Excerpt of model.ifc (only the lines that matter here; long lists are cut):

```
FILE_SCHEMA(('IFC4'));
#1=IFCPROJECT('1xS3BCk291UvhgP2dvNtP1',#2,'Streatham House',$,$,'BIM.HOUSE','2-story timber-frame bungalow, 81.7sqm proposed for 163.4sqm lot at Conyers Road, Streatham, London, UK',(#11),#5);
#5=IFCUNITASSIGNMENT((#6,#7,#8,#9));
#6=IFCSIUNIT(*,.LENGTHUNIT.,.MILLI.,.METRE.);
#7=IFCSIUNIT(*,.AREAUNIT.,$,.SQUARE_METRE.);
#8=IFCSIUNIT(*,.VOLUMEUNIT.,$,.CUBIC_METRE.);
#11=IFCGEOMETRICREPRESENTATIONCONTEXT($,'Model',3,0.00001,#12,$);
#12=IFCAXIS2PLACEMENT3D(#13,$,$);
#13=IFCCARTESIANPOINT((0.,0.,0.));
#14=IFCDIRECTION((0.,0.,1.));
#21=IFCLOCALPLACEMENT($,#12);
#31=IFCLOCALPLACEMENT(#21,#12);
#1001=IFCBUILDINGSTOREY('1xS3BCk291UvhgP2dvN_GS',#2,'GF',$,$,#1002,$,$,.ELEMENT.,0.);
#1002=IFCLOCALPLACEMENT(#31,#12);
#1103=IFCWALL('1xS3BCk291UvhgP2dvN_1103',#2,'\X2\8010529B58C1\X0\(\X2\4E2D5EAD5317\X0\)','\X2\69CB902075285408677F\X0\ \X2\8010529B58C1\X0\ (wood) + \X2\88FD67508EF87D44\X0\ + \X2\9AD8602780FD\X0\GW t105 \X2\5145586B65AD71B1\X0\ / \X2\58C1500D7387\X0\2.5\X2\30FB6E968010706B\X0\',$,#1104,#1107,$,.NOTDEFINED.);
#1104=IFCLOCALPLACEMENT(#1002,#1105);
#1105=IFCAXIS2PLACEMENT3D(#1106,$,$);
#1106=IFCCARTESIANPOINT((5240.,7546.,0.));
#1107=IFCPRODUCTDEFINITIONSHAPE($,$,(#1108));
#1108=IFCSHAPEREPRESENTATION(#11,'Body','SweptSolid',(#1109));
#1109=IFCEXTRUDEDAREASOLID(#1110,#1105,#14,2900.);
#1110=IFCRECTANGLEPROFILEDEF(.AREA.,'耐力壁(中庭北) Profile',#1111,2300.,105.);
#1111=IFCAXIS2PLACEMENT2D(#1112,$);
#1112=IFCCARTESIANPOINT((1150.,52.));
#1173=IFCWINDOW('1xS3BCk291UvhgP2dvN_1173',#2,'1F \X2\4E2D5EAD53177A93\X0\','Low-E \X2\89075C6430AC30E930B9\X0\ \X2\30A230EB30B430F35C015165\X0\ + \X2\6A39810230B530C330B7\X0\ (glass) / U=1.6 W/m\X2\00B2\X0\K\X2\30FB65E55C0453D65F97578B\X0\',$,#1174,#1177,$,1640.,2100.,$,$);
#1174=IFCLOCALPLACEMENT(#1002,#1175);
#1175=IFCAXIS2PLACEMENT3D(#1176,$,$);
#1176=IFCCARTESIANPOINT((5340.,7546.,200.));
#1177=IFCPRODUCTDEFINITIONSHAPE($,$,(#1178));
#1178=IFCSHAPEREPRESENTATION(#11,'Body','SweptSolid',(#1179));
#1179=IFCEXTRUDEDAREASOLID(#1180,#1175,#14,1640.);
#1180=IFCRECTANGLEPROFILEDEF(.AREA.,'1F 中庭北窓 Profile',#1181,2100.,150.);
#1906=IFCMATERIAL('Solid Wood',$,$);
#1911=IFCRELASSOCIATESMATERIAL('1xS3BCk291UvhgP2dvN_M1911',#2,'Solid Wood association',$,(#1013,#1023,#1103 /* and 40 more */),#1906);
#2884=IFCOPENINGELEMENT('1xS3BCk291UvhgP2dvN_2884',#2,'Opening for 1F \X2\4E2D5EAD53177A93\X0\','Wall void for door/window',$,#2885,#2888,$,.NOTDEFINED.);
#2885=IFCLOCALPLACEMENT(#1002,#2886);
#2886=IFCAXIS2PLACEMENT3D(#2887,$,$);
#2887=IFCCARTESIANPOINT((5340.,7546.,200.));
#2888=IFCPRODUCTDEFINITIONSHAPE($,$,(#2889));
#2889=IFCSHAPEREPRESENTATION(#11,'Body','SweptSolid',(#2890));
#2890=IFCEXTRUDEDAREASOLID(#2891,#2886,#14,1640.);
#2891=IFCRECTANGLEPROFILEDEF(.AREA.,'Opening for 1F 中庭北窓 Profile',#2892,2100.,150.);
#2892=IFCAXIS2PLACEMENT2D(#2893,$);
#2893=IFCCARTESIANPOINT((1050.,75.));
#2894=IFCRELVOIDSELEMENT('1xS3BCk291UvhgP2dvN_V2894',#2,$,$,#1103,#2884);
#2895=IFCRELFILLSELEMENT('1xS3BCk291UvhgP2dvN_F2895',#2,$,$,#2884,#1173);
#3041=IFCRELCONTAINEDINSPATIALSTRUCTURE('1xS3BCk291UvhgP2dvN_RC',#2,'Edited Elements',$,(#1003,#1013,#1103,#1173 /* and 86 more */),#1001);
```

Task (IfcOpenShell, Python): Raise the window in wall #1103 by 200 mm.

```python
import numpy as np
import ifcopenshell
import ifcopenshell.api.geometry
import ifcopenshell.util.placement
import ifcopenshell.util.unit

model = ifcopenshell.open("model.ifc")
unit_scale = ifcopenshell.util.unit.calculate_unit_scale(model)

window = model.by_guid("1xS3BCk291UvhgP2dvN_1173")
opening = window.FillsVoids[0].RelatingOpeningElement
dz = 0.2 / unit_scale

shift = np.array([0.0, 0.0, dz])
# The window is not placed relative to its opening, so move both.
for product in (opening, window):
    matrix = ifcopenshell.util.placement.get_local_placement(product.ObjectPlacement)
    matrix[:3, 3] += shift
    ifcopenshell.api.geometry.edit_object_placement(model, product=product, matrix=matrix, is_si=False)

print(f"moved by {dz * unit_scale:+.3f} m")

model.write("model_edited.ifc")
```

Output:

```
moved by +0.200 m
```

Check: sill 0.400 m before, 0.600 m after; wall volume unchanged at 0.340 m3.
